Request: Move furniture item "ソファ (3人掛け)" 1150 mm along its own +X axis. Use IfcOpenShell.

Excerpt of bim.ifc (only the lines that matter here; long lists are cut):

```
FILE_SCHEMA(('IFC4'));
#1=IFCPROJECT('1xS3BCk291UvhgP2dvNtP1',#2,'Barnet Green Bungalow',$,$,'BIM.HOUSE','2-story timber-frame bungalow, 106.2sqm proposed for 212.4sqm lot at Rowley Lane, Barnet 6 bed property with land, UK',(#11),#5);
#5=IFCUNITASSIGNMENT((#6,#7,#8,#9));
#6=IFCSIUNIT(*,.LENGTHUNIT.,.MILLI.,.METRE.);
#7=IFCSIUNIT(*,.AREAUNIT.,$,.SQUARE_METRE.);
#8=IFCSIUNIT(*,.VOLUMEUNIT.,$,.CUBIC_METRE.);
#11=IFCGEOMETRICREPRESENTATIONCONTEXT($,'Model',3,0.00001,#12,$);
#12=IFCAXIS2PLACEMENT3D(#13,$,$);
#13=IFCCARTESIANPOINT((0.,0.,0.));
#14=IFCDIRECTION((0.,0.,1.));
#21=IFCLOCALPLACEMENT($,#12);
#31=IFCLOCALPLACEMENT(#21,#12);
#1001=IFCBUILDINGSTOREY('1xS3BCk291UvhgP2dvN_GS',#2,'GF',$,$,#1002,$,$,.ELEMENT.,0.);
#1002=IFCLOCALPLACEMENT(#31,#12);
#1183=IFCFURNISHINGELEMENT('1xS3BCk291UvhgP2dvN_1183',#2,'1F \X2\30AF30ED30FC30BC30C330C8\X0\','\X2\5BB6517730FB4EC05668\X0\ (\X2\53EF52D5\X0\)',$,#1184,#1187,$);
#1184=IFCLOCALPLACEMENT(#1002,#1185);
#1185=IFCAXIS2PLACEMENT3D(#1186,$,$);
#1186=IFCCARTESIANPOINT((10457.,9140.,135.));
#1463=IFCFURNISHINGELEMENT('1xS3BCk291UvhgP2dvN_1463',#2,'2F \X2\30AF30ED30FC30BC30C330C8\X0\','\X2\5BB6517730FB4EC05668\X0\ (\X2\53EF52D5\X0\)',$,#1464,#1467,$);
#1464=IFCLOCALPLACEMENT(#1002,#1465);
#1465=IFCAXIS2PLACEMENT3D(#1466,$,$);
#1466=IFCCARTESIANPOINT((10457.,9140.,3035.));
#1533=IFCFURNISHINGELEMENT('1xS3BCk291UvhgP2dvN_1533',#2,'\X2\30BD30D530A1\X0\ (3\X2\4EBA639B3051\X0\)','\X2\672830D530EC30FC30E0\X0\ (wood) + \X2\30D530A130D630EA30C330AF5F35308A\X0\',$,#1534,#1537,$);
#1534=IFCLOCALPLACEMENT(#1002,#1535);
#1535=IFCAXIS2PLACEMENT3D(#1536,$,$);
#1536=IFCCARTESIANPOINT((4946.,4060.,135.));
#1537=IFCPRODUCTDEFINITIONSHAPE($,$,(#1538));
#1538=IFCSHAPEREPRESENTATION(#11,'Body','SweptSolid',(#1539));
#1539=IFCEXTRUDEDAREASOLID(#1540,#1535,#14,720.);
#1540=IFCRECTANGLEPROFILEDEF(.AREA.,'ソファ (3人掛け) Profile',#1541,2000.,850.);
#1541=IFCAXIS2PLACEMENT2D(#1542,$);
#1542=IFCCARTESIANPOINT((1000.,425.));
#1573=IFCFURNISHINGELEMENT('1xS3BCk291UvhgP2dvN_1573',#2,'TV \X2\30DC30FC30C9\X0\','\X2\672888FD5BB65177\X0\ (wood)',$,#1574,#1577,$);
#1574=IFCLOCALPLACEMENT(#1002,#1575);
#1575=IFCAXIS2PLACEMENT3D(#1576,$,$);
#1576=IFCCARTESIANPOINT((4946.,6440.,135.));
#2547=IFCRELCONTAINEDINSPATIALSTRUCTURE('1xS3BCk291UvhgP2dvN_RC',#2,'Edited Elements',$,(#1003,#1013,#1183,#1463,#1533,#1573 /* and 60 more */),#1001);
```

```python
import ifcopenshell
import ifcopenshell.api.geometry
import ifcopenshell.util.placement

model = ifcopenshell.open("bim.ifc")

item = model.by_guid("1xS3BCk291UvhgP2dvN_1533")
matrix = ifcopenshell.util.placement.get_local_placement(item.ObjectPlacement)
matrix[:3, 3] += matrix[:3, 0] * 1150.0
ifcopenshell.api.geometry.edit_object_placement(model, product=item, matrix=matrix, is_si=False)

print(ifcopenshell.util.placement.get_local_placement(item.ObjectPlacement).round(3) + 0.0)

model.write("bim-out.ifc")
```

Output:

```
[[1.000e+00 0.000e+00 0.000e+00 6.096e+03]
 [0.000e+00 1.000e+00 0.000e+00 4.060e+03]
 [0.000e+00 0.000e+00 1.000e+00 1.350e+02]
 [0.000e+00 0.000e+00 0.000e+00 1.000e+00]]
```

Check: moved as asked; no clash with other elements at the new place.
